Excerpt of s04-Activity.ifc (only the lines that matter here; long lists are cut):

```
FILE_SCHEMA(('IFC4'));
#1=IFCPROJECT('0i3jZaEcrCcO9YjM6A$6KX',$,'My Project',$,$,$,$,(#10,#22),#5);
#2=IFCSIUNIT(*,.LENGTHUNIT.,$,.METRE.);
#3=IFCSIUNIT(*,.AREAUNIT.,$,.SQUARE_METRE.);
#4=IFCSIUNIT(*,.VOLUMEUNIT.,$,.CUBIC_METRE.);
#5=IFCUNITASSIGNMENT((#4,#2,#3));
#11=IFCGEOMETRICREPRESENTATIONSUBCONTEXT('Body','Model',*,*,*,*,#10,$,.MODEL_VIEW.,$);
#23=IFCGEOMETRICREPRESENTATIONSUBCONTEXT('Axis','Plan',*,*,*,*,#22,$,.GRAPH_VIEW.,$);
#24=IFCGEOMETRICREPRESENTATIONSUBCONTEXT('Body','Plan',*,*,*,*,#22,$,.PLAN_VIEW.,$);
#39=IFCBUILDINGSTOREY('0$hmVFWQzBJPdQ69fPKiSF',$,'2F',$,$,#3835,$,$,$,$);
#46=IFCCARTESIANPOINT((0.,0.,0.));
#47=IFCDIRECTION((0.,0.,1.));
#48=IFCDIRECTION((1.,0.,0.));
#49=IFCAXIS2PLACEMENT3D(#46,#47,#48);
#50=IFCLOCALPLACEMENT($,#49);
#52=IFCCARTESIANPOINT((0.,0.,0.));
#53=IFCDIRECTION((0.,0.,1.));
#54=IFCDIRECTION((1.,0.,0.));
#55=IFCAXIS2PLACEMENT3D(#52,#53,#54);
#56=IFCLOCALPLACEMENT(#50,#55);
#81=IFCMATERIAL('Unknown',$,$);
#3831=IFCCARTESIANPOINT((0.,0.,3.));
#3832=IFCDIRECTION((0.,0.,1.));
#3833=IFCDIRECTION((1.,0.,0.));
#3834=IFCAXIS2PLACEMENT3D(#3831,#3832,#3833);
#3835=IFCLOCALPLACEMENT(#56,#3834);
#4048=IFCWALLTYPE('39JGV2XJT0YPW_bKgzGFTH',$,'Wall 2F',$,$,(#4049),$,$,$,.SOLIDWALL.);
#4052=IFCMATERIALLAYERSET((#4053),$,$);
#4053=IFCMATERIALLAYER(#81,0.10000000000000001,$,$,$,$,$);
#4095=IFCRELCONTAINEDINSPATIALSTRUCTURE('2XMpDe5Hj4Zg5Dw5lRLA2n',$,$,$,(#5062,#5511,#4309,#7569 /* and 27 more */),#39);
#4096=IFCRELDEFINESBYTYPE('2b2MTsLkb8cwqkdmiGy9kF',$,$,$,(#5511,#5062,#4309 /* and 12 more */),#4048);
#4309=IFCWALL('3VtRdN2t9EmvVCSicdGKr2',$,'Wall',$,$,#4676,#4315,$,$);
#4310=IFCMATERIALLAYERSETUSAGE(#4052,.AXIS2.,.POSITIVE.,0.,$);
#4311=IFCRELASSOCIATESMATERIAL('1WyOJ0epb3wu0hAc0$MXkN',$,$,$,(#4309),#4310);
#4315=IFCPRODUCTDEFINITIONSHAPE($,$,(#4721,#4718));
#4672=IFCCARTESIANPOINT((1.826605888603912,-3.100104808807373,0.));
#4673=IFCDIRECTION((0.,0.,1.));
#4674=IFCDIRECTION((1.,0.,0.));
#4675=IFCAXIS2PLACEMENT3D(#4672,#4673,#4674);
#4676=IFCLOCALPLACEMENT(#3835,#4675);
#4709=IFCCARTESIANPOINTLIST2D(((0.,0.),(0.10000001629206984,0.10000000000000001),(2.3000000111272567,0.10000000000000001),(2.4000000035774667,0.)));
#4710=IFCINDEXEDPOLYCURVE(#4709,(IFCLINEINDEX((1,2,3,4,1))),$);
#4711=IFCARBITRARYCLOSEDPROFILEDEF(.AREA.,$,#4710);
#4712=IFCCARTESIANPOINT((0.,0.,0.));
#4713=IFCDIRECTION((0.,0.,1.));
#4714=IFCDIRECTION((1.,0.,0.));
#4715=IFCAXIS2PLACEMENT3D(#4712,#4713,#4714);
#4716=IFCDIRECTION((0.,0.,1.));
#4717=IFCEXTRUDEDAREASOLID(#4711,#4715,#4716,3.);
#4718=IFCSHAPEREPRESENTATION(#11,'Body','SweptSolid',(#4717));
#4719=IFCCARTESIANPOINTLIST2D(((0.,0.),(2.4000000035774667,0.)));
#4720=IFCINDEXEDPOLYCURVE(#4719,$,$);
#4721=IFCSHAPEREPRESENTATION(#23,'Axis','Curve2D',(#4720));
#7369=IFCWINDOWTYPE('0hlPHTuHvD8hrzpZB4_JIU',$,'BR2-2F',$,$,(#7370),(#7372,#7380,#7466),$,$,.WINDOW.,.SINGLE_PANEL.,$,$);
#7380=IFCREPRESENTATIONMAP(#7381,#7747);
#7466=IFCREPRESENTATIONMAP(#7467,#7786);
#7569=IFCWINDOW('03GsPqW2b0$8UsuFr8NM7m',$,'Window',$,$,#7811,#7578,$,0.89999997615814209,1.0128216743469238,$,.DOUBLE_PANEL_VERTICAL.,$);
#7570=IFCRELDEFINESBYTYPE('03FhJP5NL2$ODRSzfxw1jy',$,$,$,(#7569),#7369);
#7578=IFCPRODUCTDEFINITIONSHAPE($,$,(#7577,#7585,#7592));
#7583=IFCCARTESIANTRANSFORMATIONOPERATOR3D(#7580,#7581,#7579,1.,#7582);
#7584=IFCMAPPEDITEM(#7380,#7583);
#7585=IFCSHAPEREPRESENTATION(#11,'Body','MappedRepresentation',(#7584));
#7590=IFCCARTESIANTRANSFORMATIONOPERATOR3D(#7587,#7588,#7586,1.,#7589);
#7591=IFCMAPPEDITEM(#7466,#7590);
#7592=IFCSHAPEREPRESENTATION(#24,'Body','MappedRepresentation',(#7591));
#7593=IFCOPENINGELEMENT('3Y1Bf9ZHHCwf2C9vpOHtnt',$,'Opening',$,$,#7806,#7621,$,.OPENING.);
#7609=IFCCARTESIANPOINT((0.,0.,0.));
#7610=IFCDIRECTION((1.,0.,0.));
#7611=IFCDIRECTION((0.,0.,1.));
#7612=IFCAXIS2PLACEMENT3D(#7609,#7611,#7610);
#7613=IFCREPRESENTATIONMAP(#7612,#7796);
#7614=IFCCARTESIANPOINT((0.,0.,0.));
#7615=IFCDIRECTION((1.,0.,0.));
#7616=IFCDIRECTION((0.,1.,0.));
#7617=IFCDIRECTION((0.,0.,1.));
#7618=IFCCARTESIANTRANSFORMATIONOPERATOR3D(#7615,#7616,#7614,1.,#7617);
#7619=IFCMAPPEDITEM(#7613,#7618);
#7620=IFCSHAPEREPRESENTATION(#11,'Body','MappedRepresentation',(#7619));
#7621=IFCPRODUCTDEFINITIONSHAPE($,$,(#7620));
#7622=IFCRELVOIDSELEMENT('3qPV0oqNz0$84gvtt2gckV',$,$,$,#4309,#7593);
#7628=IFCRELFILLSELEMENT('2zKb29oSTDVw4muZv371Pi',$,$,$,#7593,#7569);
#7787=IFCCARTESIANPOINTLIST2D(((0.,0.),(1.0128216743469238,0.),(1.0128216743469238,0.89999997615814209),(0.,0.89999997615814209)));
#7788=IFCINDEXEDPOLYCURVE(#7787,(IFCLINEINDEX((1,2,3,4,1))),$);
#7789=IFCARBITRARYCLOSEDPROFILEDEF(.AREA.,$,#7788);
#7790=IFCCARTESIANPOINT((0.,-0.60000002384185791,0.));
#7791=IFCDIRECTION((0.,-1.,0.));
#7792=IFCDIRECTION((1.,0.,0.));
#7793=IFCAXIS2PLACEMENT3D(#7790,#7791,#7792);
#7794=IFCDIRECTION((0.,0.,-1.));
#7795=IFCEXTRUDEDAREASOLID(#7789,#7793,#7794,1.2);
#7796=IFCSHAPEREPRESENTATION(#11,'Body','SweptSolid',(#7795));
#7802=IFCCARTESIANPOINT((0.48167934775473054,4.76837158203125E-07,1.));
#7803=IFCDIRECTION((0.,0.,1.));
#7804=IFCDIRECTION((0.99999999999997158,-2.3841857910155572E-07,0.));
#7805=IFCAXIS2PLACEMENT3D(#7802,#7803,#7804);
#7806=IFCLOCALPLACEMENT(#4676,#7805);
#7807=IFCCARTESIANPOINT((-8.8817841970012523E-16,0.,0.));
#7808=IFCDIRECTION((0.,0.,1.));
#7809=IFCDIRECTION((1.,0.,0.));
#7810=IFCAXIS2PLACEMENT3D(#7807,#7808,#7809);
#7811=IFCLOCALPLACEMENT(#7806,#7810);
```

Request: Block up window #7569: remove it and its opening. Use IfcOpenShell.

```python
import ifcopenshell
import ifcopenshell.api.feature
import ifcopenshell.api.root
import ifcopenshell.geom
import ifcopenshell.util.shape

model = ifcopenshell.open("s04-Activity.ifc")
settings = ifcopenshell.geom.settings()


def volume(element):
    """Net volume in cubic metres, openings subtracted."""
    shape = ifcopenshell.geom.create_shape(settings, element)
    return ifcopenshell.util.shape.get_volume(shape.geometry)


window = model.by_guid("03GsPqW2b0$8UsuFr8NM7m")
opening = window.FillsVoids[0].RelatingOpeningElement
wall = opening.VoidsElements[0].RelatingBuildingElement
before = volume(wall)

ifcopenshell.api.root.remove_product(model, product=window)
ifcopenshell.api.feature.remove_feature(model, feature=opening)

after = volume(wall)

print(f"wall volume {before:.3f} -> {after:.3f} m3")

model.write("s04-Activity_edited.ifc")
```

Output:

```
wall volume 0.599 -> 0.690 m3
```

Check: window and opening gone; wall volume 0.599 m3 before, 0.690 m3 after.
